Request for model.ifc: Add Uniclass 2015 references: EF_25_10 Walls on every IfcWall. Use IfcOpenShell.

First a look at what the model holds.

```python
import ifcopenshell

model = ifcopenshell.open("model.ifc")
print(model.schema)
print("classifications:", [c.Name for c in model.by_type("IfcClassification")])
for ifc_class in ("IfcDoor", "IfcRoof", "IfcStair", "IfcWall", "IfcWindow"):
    print(ifc_class, len(model.by_type(ifc_class)))
```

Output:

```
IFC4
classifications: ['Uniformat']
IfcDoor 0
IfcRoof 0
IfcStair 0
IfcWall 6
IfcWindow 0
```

```python
import ifcopenshell
import ifcopenshell.api.classification

model = ifcopenshell.open("model.ifc")

system = ifcopenshell.api.classification.add_classification(model, classification="Uniclass 2015")

codes = {
    "IfcWall": ("EF_25_10", "Walls"),
}
for ifc_class, (code, name) in codes.items():
    products = model.by_type(ifc_class)
    ifcopenshell.api.classification.add_reference(
        model, products=products, classification=system, identification=code, name=name
    )
    print(code, len(products))

model.write("model_rev.ifc")
```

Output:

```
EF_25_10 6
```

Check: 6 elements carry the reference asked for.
